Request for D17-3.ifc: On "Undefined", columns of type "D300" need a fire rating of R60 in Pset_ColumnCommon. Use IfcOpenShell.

First a look at what the model holds.

```python
import ifcopenshell
import ifcopenshell.util.element

model = ifcopenshell.open("D17-3.ifc")
print(model.schema)
storey = next(s for s in model.by_type("IfcBuildingStorey") if s.Name == "Undefined")
columns = [e for e in ifcopenshell.util.element.get_decomposition(storey) if e.is_a("IfcColumn")]
seen = {}
for e in columns:
    element_type = ifcopenshell.util.element.get_type(e)
    key = (element_type.Name if element_type != e and element_type else None, ifcopenshell.util.element.get_pset(e, "Pset_ColumnCommon", "FireRating"))
    seen[key] = seen.get(key, 0) + 1
for (name, value), count in sorted(seen.items(), key=str):
    print(count, "x", name, "|", value)
```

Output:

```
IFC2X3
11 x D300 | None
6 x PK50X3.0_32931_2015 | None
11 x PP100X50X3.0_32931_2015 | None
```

```python
import ifcopenshell
import ifcopenshell.api.pset
import ifcopenshell.util.element

model = ifcopenshell.open("D17-3.ifc")

storey = next(s for s in model.by_type("IfcBuildingStorey") if s.Name == "Undefined")
columns = [e for e in ifcopenshell.util.element.get_decomposition(storey) if e.is_a("IfcColumn")]

count = 0
for e in columns:
    element_type = ifcopenshell.util.element.get_type(e)
    if element_type in (None, e) or element_type.Name != "D300":
        continue
    found = ifcopenshell.util.element.get_pset(e, "Pset_ColumnCommon", should_inherit=False)
    if found:
        pset = model.by_id(found["id"])
        if len(ifcopenshell.util.element.get_elements_by_pset(pset)) > 1:
            pset = ifcopenshell.api.pset.unshare_pset(model, products=[e], pset=pset)[0]
    else:
        pset = ifcopenshell.api.pset.add_pset(model, product=e, name="Pset_ColumnCommon")
    ifcopenshell.api.pset.edit_pset(model, pset=pset, properties={"FireRating": "R60"})
    count += 1

print(count, "columns updated")

model.write("D17-3_v2.ifc")
```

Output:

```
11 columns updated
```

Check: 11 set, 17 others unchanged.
